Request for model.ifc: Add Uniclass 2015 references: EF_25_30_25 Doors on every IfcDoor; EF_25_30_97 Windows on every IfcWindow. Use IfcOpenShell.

First a look at what the model holds.

```python
import ifcopenshell

model = ifcopenshell.open("model.ifc")
print(model.schema)
print("classifications:", [c.Name for c in model.by_type("IfcClassification")])
for ifc_class in ("IfcDoor", "IfcRoof", "IfcStair", "IfcWall", "IfcWindow"):
    print(ifc_class, len(model.by_type(ifc_class)))
```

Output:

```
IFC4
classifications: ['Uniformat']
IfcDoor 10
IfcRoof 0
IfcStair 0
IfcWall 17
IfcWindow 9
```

```python
import ifcopenshell
import ifcopenshell.api.classification

model = ifcopenshell.open("model.ifc")

system = ifcopenshell.api.classification.add_classification(model, classification="Uniclass 2015")

codes = {
    "IfcDoor": ("EF_25_30_25", "Doors"),
    "IfcWindow": ("EF_25_30_97", "Windows"),
}
for ifc_class, (code, name) in codes.items():
    products = model.by_type(ifc_class)
    ifcopenshell.api.classification.add_reference(
        model, products=products, classification=system, identification=code, name=name
    )
    print(code, len(products))

model.write("model_edited.ifc")
```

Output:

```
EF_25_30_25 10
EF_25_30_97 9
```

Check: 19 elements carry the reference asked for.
